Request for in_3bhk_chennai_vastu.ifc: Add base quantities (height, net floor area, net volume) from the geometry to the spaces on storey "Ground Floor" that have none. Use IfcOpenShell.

First a look at what the model holds.

```python
import ifcopenshell
import ifcopenshell.util.element
import ifcopenshell.util.unit

model = ifcopenshell.open("in_3bhk_chennai_vastu.ifc")
print(model.schema)
for unit_type in ("LENGTHUNIT", "AREAUNIT", "VOLUMEUNIT"):
    print(unit_type, ifcopenshell.util.unit.calculate_unit_scale(model, unit_type))
storey = next(s for s in model.by_type("IfcBuildingStorey") if s.Name == "Ground Floor")
spaces = [e for e in ifcopenshell.util.element.get_decomposition(storey) if e.is_a("IfcSpace")]
for e in sorted(spaces, key=lambda e: e.id()):
    print(e.id(), e.is_a(), e.Name, list(ifcopenshell.util.element.get_psets(e, qtos_only=True)), sep=" | ")
```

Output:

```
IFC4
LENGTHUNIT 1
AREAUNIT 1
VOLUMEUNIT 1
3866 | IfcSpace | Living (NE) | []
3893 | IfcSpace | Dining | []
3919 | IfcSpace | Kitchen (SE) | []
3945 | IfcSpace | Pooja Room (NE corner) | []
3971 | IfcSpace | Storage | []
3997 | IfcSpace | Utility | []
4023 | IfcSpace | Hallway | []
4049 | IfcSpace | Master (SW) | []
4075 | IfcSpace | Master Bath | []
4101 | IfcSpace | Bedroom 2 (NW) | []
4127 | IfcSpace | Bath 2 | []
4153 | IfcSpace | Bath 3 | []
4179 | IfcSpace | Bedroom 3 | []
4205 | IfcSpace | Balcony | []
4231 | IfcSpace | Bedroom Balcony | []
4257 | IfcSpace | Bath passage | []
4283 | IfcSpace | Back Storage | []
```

```python
import ifcopenshell
import ifcopenshell.api.pset
import ifcopenshell.geom
import ifcopenshell.util.element
import ifcopenshell.util.shape
import ifcopenshell.util.unit

model = ifcopenshell.open("in_3bhk_chennai_vastu.ifc")
unit_scale = ifcopenshell.util.unit.calculate_unit_scale(model)
area_scale = ifcopenshell.util.unit.calculate_unit_scale(model, "AREAUNIT")
volume_scale = ifcopenshell.util.unit.calculate_unit_scale(model, "VOLUMEUNIT")
settings = ifcopenshell.geom.settings()

storey = next(s for s in model.by_type("IfcBuildingStorey") if s.Name == "Ground Floor")
spaces = [e for e in ifcopenshell.util.element.get_decomposition(storey) if e.is_a("IfcSpace")]

for e in sorted(spaces, key=lambda e: e.id()):
    if ifcopenshell.util.element.get_psets(e, qtos_only=True, should_inherit=False):
        continue
    # Geometry comes back in metres, in the element's own axes.
    shape = ifcopenshell.geom.create_shape(settings, e)
    values = {
        "Height": ifcopenshell.util.shape.get_z(shape.geometry) / unit_scale,
        "NetFloorArea": ifcopenshell.util.shape.get_footprint_area(shape.geometry) / area_scale,
        "NetVolume": ifcopenshell.util.shape.get_volume(shape.geometry) / volume_scale,
    }
    qto = ifcopenshell.api.pset.add_qto(model, product=e, name="Qto_SpaceBaseQuantities")
    ifcopenshell.api.pset.edit_qto(model, qto=qto, properties=values)
    print(e.id(), {k: round(v, 3) for k, v in values.items()})

model.write("in_3bhk_chennai_vastu_rev.ifc")
```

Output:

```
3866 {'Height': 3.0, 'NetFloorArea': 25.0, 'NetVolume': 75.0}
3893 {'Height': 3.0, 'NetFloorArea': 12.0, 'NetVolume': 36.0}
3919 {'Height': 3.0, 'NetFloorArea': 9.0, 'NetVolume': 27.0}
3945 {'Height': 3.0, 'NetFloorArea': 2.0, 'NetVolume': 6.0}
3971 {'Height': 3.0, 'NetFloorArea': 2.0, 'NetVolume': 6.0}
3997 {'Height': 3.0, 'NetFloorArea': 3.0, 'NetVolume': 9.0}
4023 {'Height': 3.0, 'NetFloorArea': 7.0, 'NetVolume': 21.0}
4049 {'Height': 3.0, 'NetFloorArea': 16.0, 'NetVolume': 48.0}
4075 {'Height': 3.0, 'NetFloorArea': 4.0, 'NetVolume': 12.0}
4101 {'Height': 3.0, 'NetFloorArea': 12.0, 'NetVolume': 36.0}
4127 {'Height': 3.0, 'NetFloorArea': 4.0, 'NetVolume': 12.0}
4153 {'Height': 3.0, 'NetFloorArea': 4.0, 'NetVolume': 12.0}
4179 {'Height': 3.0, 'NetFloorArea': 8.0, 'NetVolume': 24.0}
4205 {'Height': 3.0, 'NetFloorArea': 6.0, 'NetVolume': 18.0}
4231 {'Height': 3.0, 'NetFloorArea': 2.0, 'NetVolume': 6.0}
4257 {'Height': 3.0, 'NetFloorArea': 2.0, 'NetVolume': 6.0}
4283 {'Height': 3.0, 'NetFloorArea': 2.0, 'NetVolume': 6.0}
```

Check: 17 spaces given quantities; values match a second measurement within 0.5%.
